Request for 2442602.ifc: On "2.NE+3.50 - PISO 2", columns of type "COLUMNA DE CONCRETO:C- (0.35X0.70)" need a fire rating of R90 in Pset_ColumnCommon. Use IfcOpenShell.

First a look at what the model holds.

```python
import ifcopenshell
import ifcopenshell.util.element

model = ifcopenshell.open("2442602.ifc")
print(model.schema)
storey = next(s for s in model.by_type("IfcBuildingStorey") if s.Name == "2.NE+3.50 - PISO 2")
columns = [e for e in ifcopenshell.util.element.get_decomposition(storey) if e.is_a("IfcColumn")]
seen = {}
for e in columns:
    element_type = ifcopenshell.util.element.get_type(e)
    key = (element_type.Name if element_type != e and element_type else None, ifcopenshell.util.element.get_pset(e, "Pset_ColumnCommon", "FireRating"))
    seen[key] = seen.get(key, 0) + 1
for (name, value), count in sorted(seen.items(), key=str):
    print(count, "x", name, "|", value)
```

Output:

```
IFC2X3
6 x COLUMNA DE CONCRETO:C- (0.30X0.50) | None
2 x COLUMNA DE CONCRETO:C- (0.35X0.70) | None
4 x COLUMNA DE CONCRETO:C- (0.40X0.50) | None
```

```python
import ifcopenshell
import ifcopenshell.api.pset
import ifcopenshell.util.element

model = ifcopenshell.open("2442602.ifc")

storey = next(s for s in model.by_type("IfcBuildingStorey") if s.Name == "2.NE+3.50 - PISO 2")
columns = [e for e in ifcopenshell.util.element.get_decomposition(storey) if e.is_a("IfcColumn")]

count = 0
for e in columns:
    element_type = ifcopenshell.util.element.get_type(e)
    if element_type in (None, e) or element_type.Name != "COLUMNA DE CONCRETO:C- (0.35X0.70)":
        continue
    # add_pset returns the element's existing set when there is one.
    pset = ifcopenshell.api.pset.add_pset(model, product=e, name="Pset_ColumnCommon")
    ifcopenshell.api.pset.edit_pset(model, pset=pset, properties={"FireRating": "R90"})
    count += 1

print(count, "columns updated")

model.write("2442602-out.ifc")
```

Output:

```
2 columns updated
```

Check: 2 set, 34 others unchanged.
